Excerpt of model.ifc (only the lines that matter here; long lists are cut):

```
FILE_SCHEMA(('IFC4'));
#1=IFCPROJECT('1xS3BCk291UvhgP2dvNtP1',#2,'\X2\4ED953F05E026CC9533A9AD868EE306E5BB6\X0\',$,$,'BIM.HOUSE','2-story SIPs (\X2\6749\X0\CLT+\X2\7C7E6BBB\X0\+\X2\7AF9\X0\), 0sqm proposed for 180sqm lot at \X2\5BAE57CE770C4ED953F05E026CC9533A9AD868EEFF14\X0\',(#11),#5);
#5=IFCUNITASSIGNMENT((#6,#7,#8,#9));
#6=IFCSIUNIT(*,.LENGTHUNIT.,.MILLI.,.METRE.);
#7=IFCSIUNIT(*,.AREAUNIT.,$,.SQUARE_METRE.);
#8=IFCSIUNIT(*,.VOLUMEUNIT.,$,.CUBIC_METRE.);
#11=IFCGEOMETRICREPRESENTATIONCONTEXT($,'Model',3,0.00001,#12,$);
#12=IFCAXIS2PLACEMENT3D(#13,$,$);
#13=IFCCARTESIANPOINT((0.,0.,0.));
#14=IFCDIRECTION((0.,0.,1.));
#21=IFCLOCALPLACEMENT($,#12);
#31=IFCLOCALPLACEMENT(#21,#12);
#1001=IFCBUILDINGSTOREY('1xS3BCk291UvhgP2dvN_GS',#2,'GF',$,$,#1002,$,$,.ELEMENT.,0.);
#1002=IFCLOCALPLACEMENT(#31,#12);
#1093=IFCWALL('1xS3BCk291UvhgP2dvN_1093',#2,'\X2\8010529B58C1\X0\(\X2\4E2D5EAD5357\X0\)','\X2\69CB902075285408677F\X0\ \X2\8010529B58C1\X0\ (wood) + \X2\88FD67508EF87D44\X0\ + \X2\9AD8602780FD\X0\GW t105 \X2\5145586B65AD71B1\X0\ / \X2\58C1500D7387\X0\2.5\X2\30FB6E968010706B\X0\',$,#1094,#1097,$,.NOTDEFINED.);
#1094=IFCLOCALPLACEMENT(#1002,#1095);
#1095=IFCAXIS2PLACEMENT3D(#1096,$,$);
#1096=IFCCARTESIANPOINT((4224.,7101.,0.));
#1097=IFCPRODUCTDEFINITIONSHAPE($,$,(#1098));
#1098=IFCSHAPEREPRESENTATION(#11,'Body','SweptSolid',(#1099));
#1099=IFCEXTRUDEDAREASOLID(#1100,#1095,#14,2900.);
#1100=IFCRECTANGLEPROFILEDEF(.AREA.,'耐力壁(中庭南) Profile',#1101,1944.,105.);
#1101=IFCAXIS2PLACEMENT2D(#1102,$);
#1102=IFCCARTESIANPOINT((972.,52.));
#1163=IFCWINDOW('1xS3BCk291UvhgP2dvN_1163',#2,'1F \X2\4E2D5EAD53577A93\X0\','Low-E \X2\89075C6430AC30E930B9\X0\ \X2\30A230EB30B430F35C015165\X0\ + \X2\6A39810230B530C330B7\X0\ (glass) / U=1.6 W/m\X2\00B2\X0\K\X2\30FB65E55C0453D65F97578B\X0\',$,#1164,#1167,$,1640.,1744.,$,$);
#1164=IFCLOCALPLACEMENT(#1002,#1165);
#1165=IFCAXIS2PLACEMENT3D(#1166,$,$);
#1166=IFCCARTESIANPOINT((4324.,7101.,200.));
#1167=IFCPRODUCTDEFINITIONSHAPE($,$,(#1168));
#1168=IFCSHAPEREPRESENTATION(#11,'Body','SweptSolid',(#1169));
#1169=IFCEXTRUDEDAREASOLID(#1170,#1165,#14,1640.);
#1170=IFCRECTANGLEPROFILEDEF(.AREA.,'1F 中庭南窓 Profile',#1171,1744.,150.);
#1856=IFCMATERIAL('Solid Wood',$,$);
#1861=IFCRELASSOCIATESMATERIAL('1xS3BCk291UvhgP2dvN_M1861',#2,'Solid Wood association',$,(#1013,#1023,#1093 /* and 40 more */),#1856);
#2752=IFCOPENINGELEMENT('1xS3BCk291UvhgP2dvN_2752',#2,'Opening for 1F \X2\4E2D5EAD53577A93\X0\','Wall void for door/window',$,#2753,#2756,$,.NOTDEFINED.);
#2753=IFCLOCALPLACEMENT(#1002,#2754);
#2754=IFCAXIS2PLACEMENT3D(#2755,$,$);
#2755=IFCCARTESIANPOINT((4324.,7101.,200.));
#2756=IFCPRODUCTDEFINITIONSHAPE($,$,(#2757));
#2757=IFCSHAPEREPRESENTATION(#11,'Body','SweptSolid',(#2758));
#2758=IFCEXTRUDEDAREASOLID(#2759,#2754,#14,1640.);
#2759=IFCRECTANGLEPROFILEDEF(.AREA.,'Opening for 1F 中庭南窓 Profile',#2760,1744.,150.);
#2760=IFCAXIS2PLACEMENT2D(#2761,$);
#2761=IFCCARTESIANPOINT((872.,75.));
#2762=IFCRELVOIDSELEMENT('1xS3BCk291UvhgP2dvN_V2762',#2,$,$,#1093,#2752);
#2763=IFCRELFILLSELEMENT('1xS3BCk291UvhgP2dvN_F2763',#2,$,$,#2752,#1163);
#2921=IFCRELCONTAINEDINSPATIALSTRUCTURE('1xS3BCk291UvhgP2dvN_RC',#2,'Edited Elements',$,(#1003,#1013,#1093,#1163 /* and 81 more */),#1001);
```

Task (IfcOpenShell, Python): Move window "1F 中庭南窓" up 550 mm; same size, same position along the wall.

```python
import numpy as np
import ifcopenshell
import ifcopenshell.api.geometry
import ifcopenshell.util.placement
import ifcopenshell.util.unit

model = ifcopenshell.open("model.ifc")
unit_scale = ifcopenshell.util.unit.calculate_unit_scale(model)

window = model.by_guid("1xS3BCk291UvhgP2dvN_1163")
opening = window.FillsVoids[0].RelatingOpeningElement
dz = 0.55 / unit_scale

shift = np.array([0.0, 0.0, dz])
# The window is not placed relative to its opening, so move both.
for product in (opening, window):
    matrix = ifcopenshell.util.placement.get_local_placement(product.ObjectPlacement)
    matrix[:3, 3] += shift
    ifcopenshell.api.geometry.edit_object_placement(model, product=product, matrix=matrix, is_si=False)

print(f"moved by {dz * unit_scale:+.3f} m")

model.write("model_v2.ifc")
```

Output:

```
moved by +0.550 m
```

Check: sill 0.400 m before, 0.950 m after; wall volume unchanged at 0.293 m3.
